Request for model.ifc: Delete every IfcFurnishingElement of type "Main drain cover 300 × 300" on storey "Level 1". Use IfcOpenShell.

First a look at what the model holds.

```python
import ifcopenshell
import ifcopenshell.util.element

model = ifcopenshell.open("model.ifc")
print(model.schema)
storey = next(s for s in model.by_type("IfcBuildingStorey") if s.Name == "Level 1")
furniture = [e for e in ifcopenshell.util.element.get_decomposition(storey) if e.is_a("IfcFurnishingElement")]
seen = {}
for e in furniture:
    element_type = ifcopenshell.util.element.get_type(e)
    name = element_type.Name if element_type not in (None, e) else None
    seen[name] = seen.get(name, 0) + 1
for name, count in sorted(seen.items(), key=str):
    print(count, "x", name)
```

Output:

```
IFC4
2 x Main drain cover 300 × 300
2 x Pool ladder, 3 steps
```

```python
import ifcopenshell
import ifcopenshell.api.root
import ifcopenshell.util.element

model = ifcopenshell.open("model.ifc")

storey = next(s for s in model.by_type("IfcBuildingStorey") if s.Name == "Level 1")
furniture = [e for e in ifcopenshell.util.element.get_decomposition(storey) if e.is_a("IfcFurnishingElement")]
targets = [e for e in furniture if (t := ifcopenshell.util.element.get_type(e)) not in (None, e) and t.Name == "Main drain cover 300 × 300"]

for e in targets:
    ifcopenshell.api.root.remove_product(model, product=e)
print(len(targets), "removed")

model.write("model_edited.ifc")
```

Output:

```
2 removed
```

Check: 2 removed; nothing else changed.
